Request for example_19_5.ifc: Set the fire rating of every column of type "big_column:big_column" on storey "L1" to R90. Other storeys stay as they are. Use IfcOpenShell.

First a look at what the model holds.

```python
import ifcopenshell
import ifcopenshell.util.element

model = ifcopenshell.open("example_19_5.ifc")
print(model.schema)
storey = next(s for s in model.by_type("IfcBuildingStorey") if s.Name == "L1")
columns = [e for e in ifcopenshell.util.element.get_decomposition(storey) if e.is_a("IfcColumn")]
seen = {}
for e in columns:
    element_type = ifcopenshell.util.element.get_type(e)
    key = (element_type.Name if element_type != e and element_type else None, ifcopenshell.util.element.get_pset(e, "Pset_ColumnCommon", "FireRating"))
    seen[key] = seen.get(key, 0) + 1
for (name, value), count in sorted(seen.items(), key=str):
    print(count, "x", name, "|", value)
```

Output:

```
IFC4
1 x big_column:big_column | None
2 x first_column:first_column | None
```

```python
import ifcopenshell
import ifcopenshell.api.pset
import ifcopenshell.util.element

model = ifcopenshell.open("example_19_5.ifc")

storey = next(s for s in model.by_type("IfcBuildingStorey") if s.Name == "L1")
columns = [e for e in ifcopenshell.util.element.get_decomposition(storey) if e.is_a("IfcColumn")]

count = 0
for e in columns:
    element_type = ifcopenshell.util.element.get_type(e)
    if element_type in (None, e) or element_type.Name != "big_column:big_column":
        continue
    # add_pset returns the element's existing set when there is one.
    pset = ifcopenshell.api.pset.add_pset(model, product=e, name="Pset_ColumnCommon")
    ifcopenshell.api.pset.edit_pset(model, pset=pset, properties={"FireRating": "R90"})
    count += 1

print(count, "columns updated")

model.write("example_19_5_updated.ifc")
```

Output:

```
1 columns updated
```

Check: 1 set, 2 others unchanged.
